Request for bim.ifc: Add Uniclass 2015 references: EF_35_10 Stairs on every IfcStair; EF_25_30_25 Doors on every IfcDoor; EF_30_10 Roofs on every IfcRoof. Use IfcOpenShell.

First a look at what the model holds.

```python
import ifcopenshell

model = ifcopenshell.open("bim.ifc")
print(model.schema)
print("classifications:", [c.Name for c in model.by_type("IfcClassification")])
for ifc_class in ("IfcDoor", "IfcRoof", "IfcStair", "IfcWall", "IfcWindow"):
    print(ifc_class, len(model.by_type(ifc_class)))
```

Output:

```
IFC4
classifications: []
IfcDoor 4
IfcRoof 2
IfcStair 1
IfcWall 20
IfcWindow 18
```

```python
import ifcopenshell
import ifcopenshell.api.classification

model = ifcopenshell.open("bim.ifc")

system = ifcopenshell.api.classification.add_classification(model, classification="Uniclass 2015")

codes = {
    "IfcStair": ("EF_35_10", "Stairs"),
    "IfcDoor": ("EF_25_30_25", "Doors"),
    "IfcRoof": ("EF_30_10", "Roofs"),
}
for ifc_class, (code, name) in codes.items():
    products = model.by_type(ifc_class)
    ifcopenshell.api.classification.add_reference(
        model, products=products, classification=system, identification=code, name=name
    )
    print(code, len(products))

model.write("bim-out.ifc")
```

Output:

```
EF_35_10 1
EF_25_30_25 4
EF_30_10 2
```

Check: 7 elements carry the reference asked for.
